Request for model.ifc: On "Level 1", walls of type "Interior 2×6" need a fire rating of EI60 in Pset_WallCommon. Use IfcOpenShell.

First a look at what the model holds.

```python
import ifcopenshell
import ifcopenshell.util.element

model = ifcopenshell.open("model.ifc")
print(model.schema)
storey = next(s for s in model.by_type("IfcBuildingStorey") if s.Name == "Level 1")
walls = [e for e in ifcopenshell.util.element.get_decomposition(storey) if e.is_a("IfcWall")]
seen = {}
for e in walls:
    element_type = ifcopenshell.util.element.get_type(e)
    key = (element_type.Name if element_type != e and element_type else None, ifcopenshell.util.element.get_pset(e, "Pset_WallCommon", "FireRating"))
    seen[key] = seen.get(key, 0) + 1
for (name, value), count in sorted(seen.items(), key=str):
    print(count, "x", name, "|", value)
```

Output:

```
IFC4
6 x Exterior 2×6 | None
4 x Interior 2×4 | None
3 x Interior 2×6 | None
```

```python
import ifcopenshell
import ifcopenshell.api.pset
import ifcopenshell.util.element

model = ifcopenshell.open("model.ifc")

storey = next(s for s in model.by_type("IfcBuildingStorey") if s.Name == "Level 1")
walls = [e for e in ifcopenshell.util.element.get_decomposition(storey) if e.is_a("IfcWall")]

count = 0
for e in walls:
    element_type = ifcopenshell.util.element.get_type(e)
    if element_type in (None, e) or element_type.Name != "Interior 2×6":
        continue
    # add_pset returns the element's existing set when there is one.
    pset = ifcopenshell.api.pset.add_pset(model, product=e, name="Pset_WallCommon")
    ifcopenshell.api.pset.edit_pset(model, pset=pset, properties={"FireRating": "EI60"})
    count += 1

print(count, "walls updated")

model.write("model-out.ifc")
```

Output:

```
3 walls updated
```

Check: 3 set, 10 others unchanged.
